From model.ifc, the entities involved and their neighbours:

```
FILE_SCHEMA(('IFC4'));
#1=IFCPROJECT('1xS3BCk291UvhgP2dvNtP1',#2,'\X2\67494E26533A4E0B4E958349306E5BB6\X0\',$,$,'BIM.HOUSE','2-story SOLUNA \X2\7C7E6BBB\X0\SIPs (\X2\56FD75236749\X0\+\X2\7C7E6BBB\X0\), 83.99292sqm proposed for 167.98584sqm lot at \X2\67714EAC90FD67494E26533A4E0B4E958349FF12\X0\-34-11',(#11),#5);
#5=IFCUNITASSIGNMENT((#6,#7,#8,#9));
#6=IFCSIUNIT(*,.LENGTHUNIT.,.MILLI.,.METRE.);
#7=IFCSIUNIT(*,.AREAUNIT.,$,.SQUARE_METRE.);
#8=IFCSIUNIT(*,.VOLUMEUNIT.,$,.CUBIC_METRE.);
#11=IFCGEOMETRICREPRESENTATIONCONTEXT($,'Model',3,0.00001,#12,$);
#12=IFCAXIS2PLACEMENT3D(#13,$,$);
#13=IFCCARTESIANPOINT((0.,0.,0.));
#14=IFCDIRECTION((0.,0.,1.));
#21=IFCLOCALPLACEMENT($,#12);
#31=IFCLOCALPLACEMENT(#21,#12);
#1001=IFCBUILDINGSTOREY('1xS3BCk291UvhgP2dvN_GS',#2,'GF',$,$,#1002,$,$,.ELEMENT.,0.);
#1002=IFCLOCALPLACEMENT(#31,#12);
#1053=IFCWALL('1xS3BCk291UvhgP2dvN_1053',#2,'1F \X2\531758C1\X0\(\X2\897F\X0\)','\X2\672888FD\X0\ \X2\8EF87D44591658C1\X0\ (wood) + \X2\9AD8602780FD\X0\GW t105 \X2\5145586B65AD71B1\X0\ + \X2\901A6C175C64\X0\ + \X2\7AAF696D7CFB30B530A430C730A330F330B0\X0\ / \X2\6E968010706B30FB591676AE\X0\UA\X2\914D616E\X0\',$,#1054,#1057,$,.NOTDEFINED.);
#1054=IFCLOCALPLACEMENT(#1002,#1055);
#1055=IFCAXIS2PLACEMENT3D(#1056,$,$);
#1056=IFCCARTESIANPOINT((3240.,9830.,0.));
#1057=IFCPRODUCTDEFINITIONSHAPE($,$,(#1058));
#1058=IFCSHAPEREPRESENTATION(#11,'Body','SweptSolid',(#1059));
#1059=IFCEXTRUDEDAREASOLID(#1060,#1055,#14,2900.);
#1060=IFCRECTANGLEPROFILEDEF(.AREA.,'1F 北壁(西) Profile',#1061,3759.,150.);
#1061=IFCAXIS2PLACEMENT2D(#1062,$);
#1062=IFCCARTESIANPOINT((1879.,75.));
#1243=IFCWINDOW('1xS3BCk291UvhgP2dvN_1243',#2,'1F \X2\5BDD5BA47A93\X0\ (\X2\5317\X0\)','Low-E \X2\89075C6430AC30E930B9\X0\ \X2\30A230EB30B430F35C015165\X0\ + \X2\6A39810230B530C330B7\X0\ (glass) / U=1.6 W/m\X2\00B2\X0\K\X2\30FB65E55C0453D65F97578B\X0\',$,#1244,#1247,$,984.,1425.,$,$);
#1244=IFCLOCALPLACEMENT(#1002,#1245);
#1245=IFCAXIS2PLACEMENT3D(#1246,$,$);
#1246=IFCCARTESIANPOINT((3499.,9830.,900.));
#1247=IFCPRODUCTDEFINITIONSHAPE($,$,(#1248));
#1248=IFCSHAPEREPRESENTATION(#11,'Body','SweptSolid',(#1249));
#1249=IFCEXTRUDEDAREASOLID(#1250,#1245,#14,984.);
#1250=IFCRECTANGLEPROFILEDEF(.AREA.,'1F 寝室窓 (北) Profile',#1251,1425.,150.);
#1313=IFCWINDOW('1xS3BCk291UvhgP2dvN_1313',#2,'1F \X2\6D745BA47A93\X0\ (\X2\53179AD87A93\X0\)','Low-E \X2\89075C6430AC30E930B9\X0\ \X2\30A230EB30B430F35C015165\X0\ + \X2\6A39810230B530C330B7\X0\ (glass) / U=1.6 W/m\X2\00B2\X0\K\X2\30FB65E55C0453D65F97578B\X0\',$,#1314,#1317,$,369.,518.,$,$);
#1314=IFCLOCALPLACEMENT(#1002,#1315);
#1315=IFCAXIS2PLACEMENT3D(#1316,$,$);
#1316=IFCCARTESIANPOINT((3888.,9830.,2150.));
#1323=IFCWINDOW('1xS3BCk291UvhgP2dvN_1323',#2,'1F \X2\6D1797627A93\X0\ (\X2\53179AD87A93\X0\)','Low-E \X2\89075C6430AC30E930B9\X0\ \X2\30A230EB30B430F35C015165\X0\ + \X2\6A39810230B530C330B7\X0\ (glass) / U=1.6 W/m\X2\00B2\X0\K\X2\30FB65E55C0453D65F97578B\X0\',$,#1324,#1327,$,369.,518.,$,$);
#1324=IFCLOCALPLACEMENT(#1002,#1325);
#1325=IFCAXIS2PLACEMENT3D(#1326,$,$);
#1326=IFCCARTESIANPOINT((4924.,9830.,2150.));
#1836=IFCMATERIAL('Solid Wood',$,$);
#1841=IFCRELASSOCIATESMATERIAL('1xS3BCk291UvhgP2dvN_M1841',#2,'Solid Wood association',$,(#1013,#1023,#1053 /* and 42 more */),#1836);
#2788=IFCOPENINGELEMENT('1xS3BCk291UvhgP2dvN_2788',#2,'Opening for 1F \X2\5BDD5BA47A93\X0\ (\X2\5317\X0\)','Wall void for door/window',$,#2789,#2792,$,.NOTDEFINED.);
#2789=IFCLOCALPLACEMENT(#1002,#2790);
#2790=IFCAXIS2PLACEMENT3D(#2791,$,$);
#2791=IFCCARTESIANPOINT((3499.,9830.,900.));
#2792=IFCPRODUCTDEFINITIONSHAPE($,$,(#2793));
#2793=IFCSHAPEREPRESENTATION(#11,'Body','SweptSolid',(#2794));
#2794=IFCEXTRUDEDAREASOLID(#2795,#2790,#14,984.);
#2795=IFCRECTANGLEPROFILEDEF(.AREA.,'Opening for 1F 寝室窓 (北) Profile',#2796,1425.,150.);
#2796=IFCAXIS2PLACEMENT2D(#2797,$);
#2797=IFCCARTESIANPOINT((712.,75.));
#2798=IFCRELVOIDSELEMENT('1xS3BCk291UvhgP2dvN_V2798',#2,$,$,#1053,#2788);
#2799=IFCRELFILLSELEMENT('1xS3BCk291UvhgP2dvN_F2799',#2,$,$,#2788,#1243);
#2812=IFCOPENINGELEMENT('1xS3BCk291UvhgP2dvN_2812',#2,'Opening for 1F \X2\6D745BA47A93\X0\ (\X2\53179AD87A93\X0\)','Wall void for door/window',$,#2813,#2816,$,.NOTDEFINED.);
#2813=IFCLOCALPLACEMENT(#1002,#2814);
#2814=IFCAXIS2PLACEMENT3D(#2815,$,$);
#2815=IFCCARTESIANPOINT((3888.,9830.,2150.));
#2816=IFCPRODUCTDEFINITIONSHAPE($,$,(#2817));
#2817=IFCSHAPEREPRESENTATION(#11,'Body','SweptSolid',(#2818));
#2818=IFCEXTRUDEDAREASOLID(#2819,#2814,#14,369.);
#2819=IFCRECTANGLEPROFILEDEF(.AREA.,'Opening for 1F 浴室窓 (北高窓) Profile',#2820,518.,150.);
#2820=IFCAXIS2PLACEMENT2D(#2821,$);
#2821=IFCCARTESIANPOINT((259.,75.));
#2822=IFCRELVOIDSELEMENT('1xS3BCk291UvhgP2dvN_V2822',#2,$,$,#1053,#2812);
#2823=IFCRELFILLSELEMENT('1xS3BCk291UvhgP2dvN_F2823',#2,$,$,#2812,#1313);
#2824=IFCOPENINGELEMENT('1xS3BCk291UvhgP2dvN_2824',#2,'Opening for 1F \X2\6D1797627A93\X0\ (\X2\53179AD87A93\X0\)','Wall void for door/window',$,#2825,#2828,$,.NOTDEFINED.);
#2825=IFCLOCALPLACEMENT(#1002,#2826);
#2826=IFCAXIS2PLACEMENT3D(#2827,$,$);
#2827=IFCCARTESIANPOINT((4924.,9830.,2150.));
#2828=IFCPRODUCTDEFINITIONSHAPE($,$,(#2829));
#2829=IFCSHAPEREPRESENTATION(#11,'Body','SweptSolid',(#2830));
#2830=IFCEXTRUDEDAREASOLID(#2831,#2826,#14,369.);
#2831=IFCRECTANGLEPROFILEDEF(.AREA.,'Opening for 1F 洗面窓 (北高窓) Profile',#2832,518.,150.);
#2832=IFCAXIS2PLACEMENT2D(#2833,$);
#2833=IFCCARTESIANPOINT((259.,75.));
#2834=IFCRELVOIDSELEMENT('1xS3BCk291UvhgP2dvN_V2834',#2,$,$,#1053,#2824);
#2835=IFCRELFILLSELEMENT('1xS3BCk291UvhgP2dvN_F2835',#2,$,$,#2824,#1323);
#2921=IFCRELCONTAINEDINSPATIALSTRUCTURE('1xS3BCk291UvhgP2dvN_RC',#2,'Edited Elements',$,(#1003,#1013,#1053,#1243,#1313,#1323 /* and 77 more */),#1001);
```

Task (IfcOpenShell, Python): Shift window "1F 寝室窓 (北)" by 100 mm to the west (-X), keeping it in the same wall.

```python
import ifcopenshell
import ifcopenshell.api.geometry
import ifcopenshell.util.placement

model = ifcopenshell.open("model.ifc")

window = model.by_id(1243)
opening = window.FillsVoids[0].RelatingOpeningElement
wall = opening.VoidsElements[0].RelatingBuildingElement

wall_matrix = ifcopenshell.util.placement.get_local_placement(wall.ObjectPlacement)
shift = wall_matrix[:3, 0] * -100.0
before = ifcopenshell.util.placement.get_local_placement(window.ObjectPlacement)[:3, 3].copy()

# The window is not placed relative to its opening, so move both.
for product in (opening, window):
    matrix = ifcopenshell.util.placement.get_local_placement(product.ObjectPlacement)
    matrix[:3, 3] += shift
    ifcopenshell.api.geometry.edit_object_placement(model, product=product, matrix=matrix, is_si=False)

after = ifcopenshell.util.placement.get_local_placement(window.ObjectPlacement)[:3, 3]
print("window moved by", (after - before).round(3) + 0.0)

model.write("model_updated.ifc")
```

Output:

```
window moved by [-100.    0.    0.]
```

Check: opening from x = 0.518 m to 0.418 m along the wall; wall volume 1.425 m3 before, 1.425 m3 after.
